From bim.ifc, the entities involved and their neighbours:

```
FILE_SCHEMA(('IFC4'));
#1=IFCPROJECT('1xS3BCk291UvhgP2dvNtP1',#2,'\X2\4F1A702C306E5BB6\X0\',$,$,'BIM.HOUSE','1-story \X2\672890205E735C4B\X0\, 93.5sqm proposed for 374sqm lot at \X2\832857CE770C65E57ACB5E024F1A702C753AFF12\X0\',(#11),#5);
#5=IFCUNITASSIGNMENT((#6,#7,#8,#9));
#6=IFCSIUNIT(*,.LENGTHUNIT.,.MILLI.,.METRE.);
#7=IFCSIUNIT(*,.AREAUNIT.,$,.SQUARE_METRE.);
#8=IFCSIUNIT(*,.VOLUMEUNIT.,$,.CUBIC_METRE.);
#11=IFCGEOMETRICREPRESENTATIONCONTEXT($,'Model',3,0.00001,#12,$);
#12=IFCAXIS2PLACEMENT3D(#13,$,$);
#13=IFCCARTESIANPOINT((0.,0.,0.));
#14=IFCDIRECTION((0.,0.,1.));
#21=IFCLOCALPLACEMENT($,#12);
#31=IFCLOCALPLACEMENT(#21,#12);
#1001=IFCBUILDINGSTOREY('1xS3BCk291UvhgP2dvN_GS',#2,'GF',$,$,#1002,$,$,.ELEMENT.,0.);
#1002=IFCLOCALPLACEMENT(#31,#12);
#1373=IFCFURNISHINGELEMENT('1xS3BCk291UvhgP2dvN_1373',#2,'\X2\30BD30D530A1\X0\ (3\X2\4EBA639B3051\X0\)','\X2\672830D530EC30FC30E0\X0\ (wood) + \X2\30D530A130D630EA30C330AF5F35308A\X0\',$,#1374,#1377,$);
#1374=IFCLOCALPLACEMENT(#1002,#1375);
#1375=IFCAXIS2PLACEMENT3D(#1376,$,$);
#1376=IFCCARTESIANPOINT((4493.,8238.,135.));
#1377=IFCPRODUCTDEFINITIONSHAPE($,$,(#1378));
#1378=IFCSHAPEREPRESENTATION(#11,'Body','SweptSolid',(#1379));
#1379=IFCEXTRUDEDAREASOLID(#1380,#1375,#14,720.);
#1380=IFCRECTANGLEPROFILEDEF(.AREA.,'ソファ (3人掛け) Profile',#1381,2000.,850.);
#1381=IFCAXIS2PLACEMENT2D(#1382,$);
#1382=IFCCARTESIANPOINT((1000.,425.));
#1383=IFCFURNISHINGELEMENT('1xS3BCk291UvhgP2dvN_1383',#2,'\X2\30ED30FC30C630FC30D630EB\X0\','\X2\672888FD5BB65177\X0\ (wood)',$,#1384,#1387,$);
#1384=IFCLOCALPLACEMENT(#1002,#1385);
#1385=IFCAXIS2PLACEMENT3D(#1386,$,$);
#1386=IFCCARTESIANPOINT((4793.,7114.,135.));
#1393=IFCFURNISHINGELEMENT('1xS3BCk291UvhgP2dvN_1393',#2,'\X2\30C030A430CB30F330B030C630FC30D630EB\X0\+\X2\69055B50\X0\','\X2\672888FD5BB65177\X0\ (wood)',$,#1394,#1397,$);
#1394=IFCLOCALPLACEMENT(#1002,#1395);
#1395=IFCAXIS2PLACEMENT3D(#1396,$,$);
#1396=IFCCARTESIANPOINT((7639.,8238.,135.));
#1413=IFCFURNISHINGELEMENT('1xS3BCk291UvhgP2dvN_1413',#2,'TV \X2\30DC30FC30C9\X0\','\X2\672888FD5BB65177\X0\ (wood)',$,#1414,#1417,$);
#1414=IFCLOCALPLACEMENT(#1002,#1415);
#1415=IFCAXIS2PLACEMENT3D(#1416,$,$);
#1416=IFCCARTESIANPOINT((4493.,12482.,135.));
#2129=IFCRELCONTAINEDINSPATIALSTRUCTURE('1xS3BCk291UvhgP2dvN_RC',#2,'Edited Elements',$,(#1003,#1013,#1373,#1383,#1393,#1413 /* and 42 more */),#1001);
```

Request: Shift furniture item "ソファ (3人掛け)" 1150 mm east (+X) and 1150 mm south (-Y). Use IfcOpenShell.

```python
import ifcopenshell
import ifcopenshell.api.geometry
import ifcopenshell.util.placement
import ifcopenshell.util.unit

model = ifcopenshell.open("bim.ifc")
unit_scale = ifcopenshell.util.unit.calculate_unit_scale(model)

item = model.by_id(1373)
matrix = ifcopenshell.util.placement.get_local_placement(item.ObjectPlacement)
matrix[0, 3] += 1.15 / unit_scale
matrix[1, 3] -= 1.15 / unit_scale
ifcopenshell.api.geometry.edit_object_placement(model, product=item, matrix=matrix, is_si=False)

print(ifcopenshell.util.placement.get_local_placement(item.ObjectPlacement).round(3) + 0.0)

model.write("bim-out.ifc")
```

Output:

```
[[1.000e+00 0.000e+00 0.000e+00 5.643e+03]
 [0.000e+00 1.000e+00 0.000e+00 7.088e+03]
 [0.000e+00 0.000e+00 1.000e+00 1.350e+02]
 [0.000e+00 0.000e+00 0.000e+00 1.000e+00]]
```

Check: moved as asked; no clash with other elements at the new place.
